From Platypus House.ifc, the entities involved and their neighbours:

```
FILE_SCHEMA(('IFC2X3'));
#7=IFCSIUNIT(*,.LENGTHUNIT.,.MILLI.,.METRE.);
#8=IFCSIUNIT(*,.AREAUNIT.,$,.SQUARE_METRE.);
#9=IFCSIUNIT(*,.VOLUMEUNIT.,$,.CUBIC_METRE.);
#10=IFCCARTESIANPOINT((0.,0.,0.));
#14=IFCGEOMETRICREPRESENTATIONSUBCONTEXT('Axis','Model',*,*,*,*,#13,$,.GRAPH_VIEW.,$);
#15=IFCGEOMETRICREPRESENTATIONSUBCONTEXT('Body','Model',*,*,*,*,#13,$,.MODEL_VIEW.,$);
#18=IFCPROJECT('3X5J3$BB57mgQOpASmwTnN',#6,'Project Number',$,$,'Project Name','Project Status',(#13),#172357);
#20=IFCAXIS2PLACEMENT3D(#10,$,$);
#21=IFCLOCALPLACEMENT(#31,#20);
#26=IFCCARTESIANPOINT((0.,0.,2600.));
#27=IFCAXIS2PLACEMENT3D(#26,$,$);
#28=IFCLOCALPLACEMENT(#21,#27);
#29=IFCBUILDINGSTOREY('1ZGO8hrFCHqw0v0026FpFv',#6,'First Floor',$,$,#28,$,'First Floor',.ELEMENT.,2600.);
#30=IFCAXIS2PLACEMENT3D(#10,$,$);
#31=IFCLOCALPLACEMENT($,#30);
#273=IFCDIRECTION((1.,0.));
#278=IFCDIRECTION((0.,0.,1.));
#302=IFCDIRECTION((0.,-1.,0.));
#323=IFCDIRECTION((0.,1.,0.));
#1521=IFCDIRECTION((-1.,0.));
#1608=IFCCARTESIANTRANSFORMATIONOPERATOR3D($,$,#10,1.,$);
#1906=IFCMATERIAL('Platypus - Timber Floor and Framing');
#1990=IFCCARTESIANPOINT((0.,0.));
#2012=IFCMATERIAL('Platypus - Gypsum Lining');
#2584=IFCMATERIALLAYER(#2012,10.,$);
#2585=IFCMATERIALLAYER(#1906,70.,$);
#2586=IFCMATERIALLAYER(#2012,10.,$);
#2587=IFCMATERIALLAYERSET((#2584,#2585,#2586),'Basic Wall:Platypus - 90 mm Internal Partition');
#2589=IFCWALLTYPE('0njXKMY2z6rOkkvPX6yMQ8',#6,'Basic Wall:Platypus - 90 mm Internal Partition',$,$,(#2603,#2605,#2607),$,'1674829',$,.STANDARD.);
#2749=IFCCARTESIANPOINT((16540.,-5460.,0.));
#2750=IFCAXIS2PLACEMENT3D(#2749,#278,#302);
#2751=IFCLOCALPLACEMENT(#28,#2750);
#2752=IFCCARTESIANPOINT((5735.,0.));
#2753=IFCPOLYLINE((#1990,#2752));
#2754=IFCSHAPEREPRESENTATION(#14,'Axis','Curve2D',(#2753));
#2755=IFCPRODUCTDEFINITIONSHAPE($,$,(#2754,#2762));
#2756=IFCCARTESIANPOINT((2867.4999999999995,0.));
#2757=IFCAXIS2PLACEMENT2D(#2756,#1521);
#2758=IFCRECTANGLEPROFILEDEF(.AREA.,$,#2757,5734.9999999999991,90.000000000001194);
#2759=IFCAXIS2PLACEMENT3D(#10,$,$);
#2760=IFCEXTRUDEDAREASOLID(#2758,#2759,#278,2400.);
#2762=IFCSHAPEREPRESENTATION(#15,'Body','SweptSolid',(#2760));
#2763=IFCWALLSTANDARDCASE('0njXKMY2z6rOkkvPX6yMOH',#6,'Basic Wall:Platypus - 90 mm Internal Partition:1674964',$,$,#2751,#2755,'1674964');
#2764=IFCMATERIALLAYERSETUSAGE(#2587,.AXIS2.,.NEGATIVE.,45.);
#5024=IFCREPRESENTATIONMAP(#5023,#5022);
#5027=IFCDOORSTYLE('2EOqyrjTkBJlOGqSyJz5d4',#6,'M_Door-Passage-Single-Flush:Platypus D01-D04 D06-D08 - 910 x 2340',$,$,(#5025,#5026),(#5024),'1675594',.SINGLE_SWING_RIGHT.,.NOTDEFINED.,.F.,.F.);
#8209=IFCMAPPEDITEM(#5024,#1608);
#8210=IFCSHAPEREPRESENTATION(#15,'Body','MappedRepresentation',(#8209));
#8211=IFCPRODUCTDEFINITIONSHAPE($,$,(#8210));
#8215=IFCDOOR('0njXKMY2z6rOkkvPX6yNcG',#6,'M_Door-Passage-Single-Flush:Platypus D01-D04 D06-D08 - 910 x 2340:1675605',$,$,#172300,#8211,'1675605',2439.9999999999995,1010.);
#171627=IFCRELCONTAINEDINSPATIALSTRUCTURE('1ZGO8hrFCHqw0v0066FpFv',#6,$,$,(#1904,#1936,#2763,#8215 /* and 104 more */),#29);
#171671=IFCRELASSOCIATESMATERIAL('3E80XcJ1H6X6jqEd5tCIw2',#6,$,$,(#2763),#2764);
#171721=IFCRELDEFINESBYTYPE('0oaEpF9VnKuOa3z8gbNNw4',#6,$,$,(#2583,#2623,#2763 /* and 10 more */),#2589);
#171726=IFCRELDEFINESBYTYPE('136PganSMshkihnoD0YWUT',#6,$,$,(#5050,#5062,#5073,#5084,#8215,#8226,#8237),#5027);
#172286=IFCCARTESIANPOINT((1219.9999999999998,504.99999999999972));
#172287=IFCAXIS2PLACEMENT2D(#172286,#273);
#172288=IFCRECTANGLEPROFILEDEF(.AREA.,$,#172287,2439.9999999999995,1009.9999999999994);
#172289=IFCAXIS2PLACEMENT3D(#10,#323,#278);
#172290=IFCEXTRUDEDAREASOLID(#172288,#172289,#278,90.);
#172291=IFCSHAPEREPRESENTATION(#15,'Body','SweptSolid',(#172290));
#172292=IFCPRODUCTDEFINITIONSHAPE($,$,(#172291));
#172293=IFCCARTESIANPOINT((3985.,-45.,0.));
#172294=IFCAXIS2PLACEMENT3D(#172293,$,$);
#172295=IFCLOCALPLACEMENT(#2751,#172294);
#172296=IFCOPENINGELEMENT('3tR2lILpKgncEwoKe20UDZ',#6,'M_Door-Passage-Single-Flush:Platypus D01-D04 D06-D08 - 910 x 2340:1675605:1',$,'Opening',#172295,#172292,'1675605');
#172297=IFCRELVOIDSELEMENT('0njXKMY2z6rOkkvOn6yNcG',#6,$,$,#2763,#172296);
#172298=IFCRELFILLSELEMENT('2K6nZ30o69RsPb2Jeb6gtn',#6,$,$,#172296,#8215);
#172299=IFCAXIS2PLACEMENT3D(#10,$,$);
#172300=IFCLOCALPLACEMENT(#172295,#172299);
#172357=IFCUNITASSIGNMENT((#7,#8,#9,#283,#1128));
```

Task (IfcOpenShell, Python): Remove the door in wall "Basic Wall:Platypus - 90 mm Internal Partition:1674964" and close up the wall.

```python
import ifcopenshell
import ifcopenshell.api.feature
import ifcopenshell.api.root
import ifcopenshell.geom
import ifcopenshell.util.shape

model = ifcopenshell.open("Platypus House.ifc")
settings = ifcopenshell.geom.settings()


def volume(element):
    """Net volume in cubic metres, openings subtracted."""
    shape = ifcopenshell.geom.create_shape(settings, element)
    return ifcopenshell.util.shape.get_volume(shape.geometry)


door = model.by_id(8215)
opening = door.FillsVoids[0].RelatingOpeningElement
wall = opening.VoidsElements[0].RelatingBuildingElement
before = volume(wall)

ifcopenshell.api.root.remove_product(model, product=door)
ifcopenshell.api.feature.remove_feature(model, feature=opening)

after = volume(wall)

print(f"wall volume {before:.3f} -> {after:.3f} m3")

model.write("Platypus House_updated.ifc")
```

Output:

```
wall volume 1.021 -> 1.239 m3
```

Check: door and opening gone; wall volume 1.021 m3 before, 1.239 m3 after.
